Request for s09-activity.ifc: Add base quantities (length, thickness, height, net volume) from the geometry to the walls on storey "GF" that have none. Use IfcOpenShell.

First a look at what the model holds.

```python
import ifcopenshell
import ifcopenshell.util.element
import ifcopenshell.util.unit

model = ifcopenshell.open("s09-activity.ifc")
print(model.schema)
for unit_type in ("LENGTHUNIT", "AREAUNIT", "VOLUMEUNIT"):
    print(unit_type, ifcopenshell.util.unit.calculate_unit_scale(model, unit_type))
storey = next(s for s in model.by_type("IfcBuildingStorey") if s.Name == "GF")
walls = [e for e in ifcopenshell.util.element.get_decomposition(storey) if e.is_a("IfcWall")]
for e in sorted(walls, key=lambda e: e.id()):
    print(e.id(), e.is_a(), e.Name, list(ifcopenshell.util.element.get_psets(e, qtos_only=True)), sep=" | ")
```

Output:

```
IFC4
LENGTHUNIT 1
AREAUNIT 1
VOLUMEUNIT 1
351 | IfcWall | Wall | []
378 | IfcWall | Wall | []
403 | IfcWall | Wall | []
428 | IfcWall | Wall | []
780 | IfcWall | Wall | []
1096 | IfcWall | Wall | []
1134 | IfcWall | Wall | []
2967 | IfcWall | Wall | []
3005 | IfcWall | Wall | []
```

```python
import ifcopenshell
import ifcopenshell.api.pset
import ifcopenshell.geom
import ifcopenshell.util.element
import ifcopenshell.util.shape
import ifcopenshell.util.unit

model = ifcopenshell.open("s09-activity.ifc")
unit_scale = ifcopenshell.util.unit.calculate_unit_scale(model)
volume_scale = ifcopenshell.util.unit.calculate_unit_scale(model, "VOLUMEUNIT")
settings = ifcopenshell.geom.settings()

storey = next(s for s in model.by_type("IfcBuildingStorey") if s.Name == "GF")
walls = [e for e in ifcopenshell.util.element.get_decomposition(storey) if e.is_a("IfcWall")]

for e in sorted(walls, key=lambda e: e.id()):
    if ifcopenshell.util.element.get_psets(e, qtos_only=True, should_inherit=False):
        continue
    # Geometry comes back in metres, in the element's own axes.
    shape = ifcopenshell.geom.create_shape(settings, e)
    values = {
        "Length": ifcopenshell.util.shape.get_x(shape.geometry) / unit_scale,
        "Width": ifcopenshell.util.shape.get_y(shape.geometry) / unit_scale,
        "Height": ifcopenshell.util.shape.get_z(shape.geometry) / unit_scale,
        "NetVolume": ifcopenshell.util.shape.get_volume(shape.geometry) / volume_scale,
    }
    qto = ifcopenshell.api.pset.add_qto(model, product=e, name="Qto_WallBaseQuantities")
    ifcopenshell.api.pset.edit_qto(model, qto=qto, properties=values)
    print(e.id(), {k: round(v, 3) for k, v in values.items()})

model.write("s09-activity_edited.ifc")
```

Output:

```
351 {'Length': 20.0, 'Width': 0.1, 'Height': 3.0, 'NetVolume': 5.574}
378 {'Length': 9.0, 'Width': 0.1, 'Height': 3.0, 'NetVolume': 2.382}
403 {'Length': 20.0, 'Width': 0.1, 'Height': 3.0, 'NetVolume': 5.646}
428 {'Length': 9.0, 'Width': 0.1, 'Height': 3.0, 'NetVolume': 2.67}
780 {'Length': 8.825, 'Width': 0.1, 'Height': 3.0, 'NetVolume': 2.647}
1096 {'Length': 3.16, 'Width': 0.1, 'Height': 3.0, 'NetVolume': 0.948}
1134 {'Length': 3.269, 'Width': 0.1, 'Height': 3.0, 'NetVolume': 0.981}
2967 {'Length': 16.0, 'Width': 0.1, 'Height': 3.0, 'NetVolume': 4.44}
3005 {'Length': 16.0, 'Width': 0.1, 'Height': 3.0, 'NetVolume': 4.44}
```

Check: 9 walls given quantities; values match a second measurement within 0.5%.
